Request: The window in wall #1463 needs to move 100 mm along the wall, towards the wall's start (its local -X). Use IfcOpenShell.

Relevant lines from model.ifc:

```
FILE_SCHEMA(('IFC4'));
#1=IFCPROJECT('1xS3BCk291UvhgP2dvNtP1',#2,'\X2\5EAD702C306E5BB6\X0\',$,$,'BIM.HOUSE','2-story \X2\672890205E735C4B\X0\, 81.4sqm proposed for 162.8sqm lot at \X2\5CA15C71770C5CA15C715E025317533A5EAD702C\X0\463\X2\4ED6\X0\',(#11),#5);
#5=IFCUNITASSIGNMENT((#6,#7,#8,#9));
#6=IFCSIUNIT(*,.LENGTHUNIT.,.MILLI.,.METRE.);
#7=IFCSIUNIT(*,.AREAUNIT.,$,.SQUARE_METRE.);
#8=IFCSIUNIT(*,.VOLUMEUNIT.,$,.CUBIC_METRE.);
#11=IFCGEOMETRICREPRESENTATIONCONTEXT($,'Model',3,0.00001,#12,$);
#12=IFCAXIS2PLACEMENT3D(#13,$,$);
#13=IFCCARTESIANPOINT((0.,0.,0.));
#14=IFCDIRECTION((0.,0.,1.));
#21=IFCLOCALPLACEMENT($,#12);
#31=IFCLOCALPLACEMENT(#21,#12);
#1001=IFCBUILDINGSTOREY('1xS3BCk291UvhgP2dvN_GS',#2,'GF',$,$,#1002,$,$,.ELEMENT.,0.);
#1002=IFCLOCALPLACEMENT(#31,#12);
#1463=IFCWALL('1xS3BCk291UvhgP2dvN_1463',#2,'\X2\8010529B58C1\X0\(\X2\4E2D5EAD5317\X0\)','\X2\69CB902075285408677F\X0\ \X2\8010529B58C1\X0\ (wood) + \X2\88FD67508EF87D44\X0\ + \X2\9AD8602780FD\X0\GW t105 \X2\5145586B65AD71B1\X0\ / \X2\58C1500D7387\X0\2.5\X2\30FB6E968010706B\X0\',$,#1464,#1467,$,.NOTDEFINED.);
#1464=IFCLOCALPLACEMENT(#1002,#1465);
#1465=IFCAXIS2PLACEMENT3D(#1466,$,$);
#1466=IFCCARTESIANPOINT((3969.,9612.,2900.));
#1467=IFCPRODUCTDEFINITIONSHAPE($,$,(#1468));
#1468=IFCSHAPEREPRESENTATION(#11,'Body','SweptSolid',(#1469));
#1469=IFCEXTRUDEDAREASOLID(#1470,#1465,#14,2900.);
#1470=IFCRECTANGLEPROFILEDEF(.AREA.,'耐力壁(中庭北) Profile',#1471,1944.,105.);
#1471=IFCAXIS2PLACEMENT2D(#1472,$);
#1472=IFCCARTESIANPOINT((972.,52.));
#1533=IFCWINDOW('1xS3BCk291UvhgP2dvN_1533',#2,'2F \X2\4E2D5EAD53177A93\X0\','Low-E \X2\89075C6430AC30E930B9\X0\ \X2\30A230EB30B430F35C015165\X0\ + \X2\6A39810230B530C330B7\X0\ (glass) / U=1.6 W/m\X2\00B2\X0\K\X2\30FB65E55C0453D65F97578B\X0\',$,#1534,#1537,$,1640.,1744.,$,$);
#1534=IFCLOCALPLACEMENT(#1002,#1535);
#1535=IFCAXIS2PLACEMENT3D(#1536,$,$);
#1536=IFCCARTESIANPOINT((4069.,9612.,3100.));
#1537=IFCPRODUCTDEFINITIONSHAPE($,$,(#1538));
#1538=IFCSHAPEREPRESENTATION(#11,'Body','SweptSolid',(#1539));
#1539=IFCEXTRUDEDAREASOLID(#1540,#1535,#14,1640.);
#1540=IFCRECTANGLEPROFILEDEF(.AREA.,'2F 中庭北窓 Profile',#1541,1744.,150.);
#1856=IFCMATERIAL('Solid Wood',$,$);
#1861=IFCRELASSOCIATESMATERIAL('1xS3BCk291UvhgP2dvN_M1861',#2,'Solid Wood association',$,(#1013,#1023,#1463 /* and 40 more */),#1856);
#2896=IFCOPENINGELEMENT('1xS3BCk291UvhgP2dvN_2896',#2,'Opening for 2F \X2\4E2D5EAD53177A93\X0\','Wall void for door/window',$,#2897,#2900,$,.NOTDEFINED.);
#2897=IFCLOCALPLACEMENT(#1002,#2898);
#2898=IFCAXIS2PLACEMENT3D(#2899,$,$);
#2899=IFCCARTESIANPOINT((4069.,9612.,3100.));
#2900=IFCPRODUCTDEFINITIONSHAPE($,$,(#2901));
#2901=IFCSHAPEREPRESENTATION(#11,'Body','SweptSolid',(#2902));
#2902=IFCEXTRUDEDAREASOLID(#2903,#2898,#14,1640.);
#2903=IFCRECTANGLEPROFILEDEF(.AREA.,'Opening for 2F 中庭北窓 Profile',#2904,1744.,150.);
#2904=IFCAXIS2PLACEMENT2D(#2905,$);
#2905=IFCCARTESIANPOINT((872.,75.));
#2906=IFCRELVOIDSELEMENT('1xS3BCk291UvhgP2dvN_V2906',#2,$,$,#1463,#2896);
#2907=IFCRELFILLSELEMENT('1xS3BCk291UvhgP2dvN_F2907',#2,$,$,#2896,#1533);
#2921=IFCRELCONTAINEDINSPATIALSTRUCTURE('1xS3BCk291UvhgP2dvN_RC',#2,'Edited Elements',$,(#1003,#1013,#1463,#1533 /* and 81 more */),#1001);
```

```python
import ifcopenshell
import ifcopenshell.api.geometry
import ifcopenshell.util.placement
import ifcopenshell.util.unit

model = ifcopenshell.open("model.ifc")
unit_scale = ifcopenshell.util.unit.calculate_unit_scale(model)

window = model.by_guid("1xS3BCk291UvhgP2dvN_1533")
opening = window.FillsVoids[0].RelatingOpeningElement
wall = opening.VoidsElements[0].RelatingBuildingElement

wall_matrix = ifcopenshell.util.placement.get_local_placement(wall.ObjectPlacement)
shift = wall_matrix[:3, 0] * -0.1 / unit_scale
before = ifcopenshell.util.placement.get_local_placement(window.ObjectPlacement)[:3, 3].copy()

# The window is not placed relative to its opening, so move both.
for product in (opening, window):
    matrix = ifcopenshell.util.placement.get_local_placement(product.ObjectPlacement)
    matrix[:3, 3] += shift
    ifcopenshell.api.geometry.edit_object_placement(model, product=product, matrix=matrix, is_si=False)

after = ifcopenshell.util.placement.get_local_placement(window.ObjectPlacement)[:3, 3]
print("window moved by", (after - before).round(3) + 0.0)

model.write("model-out.ifc")
```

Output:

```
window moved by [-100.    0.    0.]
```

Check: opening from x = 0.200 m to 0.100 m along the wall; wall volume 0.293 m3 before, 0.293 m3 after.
